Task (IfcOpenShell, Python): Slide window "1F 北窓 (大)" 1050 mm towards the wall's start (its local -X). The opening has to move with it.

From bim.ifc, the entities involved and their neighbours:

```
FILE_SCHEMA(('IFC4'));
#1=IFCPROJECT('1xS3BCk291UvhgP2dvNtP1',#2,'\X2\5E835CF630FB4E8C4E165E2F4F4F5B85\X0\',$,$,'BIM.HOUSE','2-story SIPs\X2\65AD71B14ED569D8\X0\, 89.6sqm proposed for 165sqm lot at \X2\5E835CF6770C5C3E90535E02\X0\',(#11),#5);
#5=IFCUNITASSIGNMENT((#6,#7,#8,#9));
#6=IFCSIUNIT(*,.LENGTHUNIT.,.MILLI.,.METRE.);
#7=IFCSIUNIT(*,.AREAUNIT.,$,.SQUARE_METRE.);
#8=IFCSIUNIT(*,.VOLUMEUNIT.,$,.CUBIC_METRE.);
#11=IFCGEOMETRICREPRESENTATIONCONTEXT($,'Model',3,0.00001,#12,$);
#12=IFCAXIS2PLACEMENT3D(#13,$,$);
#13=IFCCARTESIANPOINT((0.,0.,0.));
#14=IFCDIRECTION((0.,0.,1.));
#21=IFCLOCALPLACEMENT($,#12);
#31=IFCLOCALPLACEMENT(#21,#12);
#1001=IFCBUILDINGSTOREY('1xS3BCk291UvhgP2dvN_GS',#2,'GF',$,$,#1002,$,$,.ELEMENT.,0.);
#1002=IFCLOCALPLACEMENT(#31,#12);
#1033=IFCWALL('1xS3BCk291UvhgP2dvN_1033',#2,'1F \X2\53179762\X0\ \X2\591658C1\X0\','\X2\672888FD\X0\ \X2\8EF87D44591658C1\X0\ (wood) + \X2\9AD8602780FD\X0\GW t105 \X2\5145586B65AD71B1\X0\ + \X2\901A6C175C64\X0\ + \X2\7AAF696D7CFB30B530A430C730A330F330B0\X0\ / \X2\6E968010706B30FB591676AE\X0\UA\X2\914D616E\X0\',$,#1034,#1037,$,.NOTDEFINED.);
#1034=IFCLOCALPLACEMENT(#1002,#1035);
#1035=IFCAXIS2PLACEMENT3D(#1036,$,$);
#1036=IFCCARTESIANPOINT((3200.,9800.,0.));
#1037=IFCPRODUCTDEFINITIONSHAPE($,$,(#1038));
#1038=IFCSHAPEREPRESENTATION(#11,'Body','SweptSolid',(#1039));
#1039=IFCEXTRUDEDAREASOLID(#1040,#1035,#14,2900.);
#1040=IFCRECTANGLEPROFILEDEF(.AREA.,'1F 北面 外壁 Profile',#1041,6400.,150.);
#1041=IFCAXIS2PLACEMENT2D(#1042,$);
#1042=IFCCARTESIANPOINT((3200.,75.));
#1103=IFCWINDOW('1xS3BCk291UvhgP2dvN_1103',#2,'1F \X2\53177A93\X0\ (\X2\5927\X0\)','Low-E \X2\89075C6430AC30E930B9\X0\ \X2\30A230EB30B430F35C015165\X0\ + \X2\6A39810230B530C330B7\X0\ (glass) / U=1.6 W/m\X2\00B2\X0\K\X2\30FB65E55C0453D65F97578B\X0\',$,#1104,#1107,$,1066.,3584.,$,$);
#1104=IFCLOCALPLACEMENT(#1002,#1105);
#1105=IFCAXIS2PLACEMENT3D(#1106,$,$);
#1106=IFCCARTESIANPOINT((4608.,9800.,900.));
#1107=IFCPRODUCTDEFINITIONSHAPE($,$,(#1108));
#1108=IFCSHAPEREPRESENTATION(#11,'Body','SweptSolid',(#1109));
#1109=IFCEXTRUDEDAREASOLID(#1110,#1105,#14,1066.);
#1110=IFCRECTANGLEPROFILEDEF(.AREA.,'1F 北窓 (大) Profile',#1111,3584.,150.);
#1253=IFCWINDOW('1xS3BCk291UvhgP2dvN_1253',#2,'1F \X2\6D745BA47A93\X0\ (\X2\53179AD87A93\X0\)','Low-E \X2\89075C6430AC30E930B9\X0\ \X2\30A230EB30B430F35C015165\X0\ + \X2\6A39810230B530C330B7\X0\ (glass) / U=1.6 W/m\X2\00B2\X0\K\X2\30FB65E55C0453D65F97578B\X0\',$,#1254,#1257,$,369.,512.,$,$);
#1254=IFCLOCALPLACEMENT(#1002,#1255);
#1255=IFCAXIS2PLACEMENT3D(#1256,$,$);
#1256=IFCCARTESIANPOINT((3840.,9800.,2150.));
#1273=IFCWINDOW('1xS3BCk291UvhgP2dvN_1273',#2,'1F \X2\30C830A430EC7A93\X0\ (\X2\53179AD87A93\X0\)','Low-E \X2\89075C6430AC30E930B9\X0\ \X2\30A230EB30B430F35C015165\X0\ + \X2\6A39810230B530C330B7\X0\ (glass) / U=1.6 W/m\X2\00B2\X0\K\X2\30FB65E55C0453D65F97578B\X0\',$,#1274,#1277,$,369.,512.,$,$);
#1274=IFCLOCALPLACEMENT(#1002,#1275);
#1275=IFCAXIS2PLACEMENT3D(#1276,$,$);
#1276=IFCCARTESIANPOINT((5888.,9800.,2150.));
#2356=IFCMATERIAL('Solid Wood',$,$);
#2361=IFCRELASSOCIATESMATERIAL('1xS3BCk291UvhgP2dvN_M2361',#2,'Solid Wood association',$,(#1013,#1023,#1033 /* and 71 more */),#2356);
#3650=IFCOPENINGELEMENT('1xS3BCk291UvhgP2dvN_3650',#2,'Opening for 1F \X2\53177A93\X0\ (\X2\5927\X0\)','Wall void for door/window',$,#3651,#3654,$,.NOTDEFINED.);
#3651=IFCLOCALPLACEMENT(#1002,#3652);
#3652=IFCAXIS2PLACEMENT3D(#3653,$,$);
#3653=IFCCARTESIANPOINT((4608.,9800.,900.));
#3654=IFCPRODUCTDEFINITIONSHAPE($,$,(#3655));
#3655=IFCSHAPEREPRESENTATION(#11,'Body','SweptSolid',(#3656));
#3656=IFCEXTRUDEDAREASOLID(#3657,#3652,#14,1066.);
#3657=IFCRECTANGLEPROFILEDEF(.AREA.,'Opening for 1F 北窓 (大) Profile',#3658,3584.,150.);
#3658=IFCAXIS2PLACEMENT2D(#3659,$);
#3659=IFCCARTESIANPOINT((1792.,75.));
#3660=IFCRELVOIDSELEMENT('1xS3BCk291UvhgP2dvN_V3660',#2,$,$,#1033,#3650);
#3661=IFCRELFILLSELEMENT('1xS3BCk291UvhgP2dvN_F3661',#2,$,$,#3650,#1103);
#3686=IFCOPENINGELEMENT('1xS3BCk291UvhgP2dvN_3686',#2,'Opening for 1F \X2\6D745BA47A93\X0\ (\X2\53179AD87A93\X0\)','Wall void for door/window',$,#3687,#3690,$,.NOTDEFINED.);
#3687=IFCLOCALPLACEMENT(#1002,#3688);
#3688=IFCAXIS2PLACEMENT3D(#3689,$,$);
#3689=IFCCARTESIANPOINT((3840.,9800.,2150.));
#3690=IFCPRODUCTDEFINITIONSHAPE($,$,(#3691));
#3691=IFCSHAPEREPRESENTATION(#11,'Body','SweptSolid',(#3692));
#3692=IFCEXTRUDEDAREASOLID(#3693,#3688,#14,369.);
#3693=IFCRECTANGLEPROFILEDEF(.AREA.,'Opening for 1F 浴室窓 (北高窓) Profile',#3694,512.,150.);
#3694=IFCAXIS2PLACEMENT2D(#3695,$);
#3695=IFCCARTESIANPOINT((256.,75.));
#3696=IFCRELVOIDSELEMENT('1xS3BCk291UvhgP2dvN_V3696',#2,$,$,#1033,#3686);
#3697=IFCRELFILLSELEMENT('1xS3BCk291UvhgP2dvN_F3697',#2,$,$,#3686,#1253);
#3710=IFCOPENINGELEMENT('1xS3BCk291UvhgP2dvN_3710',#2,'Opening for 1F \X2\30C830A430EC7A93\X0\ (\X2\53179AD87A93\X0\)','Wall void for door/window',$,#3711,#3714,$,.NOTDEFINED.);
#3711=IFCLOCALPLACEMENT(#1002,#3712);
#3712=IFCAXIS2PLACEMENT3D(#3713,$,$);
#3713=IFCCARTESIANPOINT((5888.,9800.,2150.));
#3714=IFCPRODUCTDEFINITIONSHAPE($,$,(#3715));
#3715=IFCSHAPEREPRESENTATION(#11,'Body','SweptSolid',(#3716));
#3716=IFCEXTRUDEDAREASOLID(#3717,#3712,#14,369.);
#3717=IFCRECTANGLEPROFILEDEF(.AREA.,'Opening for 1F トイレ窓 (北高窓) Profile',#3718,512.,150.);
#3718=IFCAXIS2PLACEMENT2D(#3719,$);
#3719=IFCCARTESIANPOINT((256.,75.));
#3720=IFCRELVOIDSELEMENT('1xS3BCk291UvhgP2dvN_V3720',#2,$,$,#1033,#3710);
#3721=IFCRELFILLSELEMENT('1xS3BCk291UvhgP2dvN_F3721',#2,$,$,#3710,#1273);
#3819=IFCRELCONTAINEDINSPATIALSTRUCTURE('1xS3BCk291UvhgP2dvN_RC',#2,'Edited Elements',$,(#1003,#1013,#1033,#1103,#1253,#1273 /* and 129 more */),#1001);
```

```python
import ifcopenshell
import ifcopenshell.api.geometry
import ifcopenshell.util.placement

model = ifcopenshell.open("bim.ifc")

window = model.by_id(1103)
opening = window.FillsVoids[0].RelatingOpeningElement
wall = opening.VoidsElements[0].RelatingBuildingElement

wall_matrix = ifcopenshell.util.placement.get_local_placement(wall.ObjectPlacement)
shift = wall_matrix[:3, 0] * -1050.0
before = ifcopenshell.util.placement.get_local_placement(window.ObjectPlacement)[:3, 3].copy()

# The window is not placed relative to its opening, so move both.
for product in (opening, window):
    matrix = ifcopenshell.util.placement.get_local_placement(product.ObjectPlacement)
    matrix[:3, 3] += shift
    ifcopenshell.api.geometry.edit_object_placement(model, product=product, matrix=matrix, is_si=False)

after = ifcopenshell.util.placement.get_local_placement(window.ObjectPlacement)[:3, 3]
print("window moved by", (after - before).round(3) + 0.0)

model.write("bim_rev.ifc")
```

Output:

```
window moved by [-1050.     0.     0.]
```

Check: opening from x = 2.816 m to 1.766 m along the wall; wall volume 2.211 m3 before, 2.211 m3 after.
